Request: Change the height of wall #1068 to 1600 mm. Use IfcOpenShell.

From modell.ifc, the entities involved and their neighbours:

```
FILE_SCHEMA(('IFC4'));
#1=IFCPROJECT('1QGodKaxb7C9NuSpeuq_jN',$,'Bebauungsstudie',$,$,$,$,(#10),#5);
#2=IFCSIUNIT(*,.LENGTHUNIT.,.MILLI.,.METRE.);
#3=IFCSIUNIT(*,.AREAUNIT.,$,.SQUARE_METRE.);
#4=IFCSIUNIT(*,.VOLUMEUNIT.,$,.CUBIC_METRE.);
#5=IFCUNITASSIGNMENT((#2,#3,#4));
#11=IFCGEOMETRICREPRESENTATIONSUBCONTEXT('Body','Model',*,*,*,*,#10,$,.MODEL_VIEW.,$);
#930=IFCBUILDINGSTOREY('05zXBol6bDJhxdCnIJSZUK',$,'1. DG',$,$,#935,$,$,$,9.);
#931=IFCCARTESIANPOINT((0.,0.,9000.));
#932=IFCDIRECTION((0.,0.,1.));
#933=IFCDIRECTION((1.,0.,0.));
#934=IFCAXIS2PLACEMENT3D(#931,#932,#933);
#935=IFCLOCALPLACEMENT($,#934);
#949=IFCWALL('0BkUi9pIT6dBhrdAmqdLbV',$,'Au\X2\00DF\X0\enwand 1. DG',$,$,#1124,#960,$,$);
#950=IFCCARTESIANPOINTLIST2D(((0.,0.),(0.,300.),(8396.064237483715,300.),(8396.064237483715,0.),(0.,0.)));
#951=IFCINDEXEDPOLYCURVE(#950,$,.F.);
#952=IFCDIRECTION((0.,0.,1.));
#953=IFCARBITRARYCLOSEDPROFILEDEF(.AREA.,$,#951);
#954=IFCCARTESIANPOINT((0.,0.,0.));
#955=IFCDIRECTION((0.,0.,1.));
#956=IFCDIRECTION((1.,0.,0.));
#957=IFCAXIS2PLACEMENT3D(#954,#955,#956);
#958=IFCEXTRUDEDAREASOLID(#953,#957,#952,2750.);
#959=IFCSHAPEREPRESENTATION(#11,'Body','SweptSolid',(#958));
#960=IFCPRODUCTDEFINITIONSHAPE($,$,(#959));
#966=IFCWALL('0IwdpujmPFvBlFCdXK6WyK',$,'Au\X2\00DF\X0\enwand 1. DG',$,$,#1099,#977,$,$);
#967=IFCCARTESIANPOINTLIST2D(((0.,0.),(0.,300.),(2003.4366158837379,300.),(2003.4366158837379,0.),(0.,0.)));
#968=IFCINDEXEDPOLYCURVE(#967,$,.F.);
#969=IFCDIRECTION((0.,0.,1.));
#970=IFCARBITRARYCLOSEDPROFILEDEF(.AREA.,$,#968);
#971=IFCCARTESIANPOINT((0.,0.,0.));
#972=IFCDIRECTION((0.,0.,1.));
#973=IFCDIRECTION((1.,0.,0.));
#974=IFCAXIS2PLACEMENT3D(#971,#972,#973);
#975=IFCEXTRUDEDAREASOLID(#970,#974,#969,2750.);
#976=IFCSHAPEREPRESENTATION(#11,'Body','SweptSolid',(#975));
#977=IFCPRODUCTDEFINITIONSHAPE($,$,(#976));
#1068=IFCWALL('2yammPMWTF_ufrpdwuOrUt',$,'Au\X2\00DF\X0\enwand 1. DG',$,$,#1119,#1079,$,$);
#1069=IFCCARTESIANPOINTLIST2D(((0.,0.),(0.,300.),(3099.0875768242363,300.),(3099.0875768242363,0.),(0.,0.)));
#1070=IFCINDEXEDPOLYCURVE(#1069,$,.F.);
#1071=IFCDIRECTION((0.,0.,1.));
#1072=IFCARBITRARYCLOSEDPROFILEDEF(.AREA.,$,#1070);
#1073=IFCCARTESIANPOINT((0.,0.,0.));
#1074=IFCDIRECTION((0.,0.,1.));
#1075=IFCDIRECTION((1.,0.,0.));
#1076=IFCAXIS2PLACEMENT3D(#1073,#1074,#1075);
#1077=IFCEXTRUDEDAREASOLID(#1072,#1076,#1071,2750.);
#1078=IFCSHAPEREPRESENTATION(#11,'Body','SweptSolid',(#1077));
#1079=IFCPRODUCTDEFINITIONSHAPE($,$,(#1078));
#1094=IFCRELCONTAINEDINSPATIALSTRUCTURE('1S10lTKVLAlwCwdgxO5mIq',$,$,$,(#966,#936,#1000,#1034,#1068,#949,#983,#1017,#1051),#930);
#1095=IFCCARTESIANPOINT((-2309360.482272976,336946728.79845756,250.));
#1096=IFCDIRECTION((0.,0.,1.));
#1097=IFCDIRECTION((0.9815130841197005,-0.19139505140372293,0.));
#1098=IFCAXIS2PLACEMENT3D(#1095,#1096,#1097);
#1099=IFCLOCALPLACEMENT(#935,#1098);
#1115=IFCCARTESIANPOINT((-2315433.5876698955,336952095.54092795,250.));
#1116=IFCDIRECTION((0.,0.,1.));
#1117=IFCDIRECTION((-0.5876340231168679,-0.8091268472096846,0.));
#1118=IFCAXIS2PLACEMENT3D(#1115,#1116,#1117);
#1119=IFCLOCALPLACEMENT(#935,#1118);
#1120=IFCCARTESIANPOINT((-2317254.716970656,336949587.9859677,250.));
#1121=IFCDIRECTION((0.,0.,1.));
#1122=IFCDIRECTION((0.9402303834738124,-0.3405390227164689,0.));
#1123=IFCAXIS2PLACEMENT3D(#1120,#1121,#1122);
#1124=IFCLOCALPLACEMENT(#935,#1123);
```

```python
import ifcopenshell
import ifcopenshell.geom
import ifcopenshell.util.representation
import ifcopenshell.util.shape
import ifcopenshell.util.unit

model = ifcopenshell.open("modell.ifc")
unit_scale = ifcopenshell.util.unit.calculate_unit_scale(model)
settings = ifcopenshell.geom.settings()


def volume(element):
    """Net volume in cubic metres, openings subtracted."""
    shape = ifcopenshell.geom.create_shape(settings, element)
    return ifcopenshell.util.shape.get_volume(shape.geometry)


wall = model.by_guid("2yammPMWTF_ufrpdwuOrUt")
before = volume(wall)

body = ifcopenshell.util.representation.get_representation(wall, "Model", "Body")
solid = body.Items[0]
old_height = solid.Depth
solid.Depth = 1.6 / unit_scale
after = volume(wall)

print(f"height {old_height:g} -> {solid.Depth:g}, volume {before:.3f} -> {after:.3f} m3")

model.write("modell_rev.ifc")
```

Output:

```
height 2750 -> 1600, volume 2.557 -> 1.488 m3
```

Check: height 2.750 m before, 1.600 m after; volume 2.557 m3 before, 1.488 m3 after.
